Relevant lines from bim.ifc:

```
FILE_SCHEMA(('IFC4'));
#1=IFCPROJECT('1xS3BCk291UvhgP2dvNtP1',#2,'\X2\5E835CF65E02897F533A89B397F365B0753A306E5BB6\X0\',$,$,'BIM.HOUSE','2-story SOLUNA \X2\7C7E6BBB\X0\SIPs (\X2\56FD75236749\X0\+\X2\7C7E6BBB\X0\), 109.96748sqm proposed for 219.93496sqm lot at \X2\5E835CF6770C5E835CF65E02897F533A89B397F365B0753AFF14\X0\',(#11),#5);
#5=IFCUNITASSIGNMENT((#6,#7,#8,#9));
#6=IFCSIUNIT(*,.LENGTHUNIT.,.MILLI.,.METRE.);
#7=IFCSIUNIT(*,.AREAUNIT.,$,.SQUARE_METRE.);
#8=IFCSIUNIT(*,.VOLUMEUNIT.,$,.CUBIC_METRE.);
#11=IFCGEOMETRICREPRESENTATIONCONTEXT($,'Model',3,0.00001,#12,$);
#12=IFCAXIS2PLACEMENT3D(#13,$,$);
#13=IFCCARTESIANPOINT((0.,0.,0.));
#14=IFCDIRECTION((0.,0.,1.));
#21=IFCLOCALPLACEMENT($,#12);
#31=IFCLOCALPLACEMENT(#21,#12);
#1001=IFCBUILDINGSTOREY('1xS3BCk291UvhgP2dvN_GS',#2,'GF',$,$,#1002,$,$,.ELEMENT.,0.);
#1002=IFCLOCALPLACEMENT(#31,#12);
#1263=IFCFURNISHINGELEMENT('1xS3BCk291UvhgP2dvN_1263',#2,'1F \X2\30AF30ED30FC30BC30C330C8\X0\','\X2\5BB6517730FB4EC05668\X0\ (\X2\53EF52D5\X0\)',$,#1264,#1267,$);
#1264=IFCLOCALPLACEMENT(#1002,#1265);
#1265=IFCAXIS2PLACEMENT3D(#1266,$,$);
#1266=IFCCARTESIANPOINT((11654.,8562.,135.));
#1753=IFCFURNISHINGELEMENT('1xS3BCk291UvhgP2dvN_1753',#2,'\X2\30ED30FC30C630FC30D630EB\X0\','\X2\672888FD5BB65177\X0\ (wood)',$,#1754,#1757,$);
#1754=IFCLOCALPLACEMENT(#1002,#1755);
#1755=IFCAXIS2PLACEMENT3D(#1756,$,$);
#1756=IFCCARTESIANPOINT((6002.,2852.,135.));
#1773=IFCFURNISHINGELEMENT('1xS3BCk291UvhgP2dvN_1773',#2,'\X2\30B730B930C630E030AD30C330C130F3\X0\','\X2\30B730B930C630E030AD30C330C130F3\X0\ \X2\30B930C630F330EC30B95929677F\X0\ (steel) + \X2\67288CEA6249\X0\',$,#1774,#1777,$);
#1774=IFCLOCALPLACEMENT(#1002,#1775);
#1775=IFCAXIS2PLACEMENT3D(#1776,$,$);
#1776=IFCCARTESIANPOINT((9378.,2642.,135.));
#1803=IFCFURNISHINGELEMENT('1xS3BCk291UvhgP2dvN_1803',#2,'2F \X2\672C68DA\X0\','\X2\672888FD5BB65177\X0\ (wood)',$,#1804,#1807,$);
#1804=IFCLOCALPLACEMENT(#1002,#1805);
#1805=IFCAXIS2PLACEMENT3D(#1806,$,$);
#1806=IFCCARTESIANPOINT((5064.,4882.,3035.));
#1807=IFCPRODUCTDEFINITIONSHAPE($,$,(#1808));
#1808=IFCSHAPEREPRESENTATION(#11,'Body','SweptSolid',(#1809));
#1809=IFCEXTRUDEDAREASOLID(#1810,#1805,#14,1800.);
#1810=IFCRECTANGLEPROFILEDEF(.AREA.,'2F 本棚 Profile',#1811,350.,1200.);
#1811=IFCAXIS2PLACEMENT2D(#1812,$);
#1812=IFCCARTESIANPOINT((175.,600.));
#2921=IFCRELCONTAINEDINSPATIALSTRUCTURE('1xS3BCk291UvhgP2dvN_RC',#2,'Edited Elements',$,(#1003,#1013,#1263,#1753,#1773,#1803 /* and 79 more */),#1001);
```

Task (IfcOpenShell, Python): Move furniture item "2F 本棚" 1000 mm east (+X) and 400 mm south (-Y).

```python
import ifcopenshell
import ifcopenshell.api.geometry
import ifcopenshell.util.placement
import ifcopenshell.util.unit

model = ifcopenshell.open("bim.ifc")
unit_scale = ifcopenshell.util.unit.calculate_unit_scale(model)

item = model.by_id(1803)
matrix = ifcopenshell.util.placement.get_local_placement(item.ObjectPlacement)
matrix[0, 3] += 1 / unit_scale
matrix[1, 3] -= 0.4 / unit_scale
ifcopenshell.api.geometry.edit_object_placement(model, product=item, matrix=matrix, is_si=False)

print(ifcopenshell.util.placement.get_local_placement(item.ObjectPlacement).round(3) + 0.0)

model.write("bim_edited.ifc")
```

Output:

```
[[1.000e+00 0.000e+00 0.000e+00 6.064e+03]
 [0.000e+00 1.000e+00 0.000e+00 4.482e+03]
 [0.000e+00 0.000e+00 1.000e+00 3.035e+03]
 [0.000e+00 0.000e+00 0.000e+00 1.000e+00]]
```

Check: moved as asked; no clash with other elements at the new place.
